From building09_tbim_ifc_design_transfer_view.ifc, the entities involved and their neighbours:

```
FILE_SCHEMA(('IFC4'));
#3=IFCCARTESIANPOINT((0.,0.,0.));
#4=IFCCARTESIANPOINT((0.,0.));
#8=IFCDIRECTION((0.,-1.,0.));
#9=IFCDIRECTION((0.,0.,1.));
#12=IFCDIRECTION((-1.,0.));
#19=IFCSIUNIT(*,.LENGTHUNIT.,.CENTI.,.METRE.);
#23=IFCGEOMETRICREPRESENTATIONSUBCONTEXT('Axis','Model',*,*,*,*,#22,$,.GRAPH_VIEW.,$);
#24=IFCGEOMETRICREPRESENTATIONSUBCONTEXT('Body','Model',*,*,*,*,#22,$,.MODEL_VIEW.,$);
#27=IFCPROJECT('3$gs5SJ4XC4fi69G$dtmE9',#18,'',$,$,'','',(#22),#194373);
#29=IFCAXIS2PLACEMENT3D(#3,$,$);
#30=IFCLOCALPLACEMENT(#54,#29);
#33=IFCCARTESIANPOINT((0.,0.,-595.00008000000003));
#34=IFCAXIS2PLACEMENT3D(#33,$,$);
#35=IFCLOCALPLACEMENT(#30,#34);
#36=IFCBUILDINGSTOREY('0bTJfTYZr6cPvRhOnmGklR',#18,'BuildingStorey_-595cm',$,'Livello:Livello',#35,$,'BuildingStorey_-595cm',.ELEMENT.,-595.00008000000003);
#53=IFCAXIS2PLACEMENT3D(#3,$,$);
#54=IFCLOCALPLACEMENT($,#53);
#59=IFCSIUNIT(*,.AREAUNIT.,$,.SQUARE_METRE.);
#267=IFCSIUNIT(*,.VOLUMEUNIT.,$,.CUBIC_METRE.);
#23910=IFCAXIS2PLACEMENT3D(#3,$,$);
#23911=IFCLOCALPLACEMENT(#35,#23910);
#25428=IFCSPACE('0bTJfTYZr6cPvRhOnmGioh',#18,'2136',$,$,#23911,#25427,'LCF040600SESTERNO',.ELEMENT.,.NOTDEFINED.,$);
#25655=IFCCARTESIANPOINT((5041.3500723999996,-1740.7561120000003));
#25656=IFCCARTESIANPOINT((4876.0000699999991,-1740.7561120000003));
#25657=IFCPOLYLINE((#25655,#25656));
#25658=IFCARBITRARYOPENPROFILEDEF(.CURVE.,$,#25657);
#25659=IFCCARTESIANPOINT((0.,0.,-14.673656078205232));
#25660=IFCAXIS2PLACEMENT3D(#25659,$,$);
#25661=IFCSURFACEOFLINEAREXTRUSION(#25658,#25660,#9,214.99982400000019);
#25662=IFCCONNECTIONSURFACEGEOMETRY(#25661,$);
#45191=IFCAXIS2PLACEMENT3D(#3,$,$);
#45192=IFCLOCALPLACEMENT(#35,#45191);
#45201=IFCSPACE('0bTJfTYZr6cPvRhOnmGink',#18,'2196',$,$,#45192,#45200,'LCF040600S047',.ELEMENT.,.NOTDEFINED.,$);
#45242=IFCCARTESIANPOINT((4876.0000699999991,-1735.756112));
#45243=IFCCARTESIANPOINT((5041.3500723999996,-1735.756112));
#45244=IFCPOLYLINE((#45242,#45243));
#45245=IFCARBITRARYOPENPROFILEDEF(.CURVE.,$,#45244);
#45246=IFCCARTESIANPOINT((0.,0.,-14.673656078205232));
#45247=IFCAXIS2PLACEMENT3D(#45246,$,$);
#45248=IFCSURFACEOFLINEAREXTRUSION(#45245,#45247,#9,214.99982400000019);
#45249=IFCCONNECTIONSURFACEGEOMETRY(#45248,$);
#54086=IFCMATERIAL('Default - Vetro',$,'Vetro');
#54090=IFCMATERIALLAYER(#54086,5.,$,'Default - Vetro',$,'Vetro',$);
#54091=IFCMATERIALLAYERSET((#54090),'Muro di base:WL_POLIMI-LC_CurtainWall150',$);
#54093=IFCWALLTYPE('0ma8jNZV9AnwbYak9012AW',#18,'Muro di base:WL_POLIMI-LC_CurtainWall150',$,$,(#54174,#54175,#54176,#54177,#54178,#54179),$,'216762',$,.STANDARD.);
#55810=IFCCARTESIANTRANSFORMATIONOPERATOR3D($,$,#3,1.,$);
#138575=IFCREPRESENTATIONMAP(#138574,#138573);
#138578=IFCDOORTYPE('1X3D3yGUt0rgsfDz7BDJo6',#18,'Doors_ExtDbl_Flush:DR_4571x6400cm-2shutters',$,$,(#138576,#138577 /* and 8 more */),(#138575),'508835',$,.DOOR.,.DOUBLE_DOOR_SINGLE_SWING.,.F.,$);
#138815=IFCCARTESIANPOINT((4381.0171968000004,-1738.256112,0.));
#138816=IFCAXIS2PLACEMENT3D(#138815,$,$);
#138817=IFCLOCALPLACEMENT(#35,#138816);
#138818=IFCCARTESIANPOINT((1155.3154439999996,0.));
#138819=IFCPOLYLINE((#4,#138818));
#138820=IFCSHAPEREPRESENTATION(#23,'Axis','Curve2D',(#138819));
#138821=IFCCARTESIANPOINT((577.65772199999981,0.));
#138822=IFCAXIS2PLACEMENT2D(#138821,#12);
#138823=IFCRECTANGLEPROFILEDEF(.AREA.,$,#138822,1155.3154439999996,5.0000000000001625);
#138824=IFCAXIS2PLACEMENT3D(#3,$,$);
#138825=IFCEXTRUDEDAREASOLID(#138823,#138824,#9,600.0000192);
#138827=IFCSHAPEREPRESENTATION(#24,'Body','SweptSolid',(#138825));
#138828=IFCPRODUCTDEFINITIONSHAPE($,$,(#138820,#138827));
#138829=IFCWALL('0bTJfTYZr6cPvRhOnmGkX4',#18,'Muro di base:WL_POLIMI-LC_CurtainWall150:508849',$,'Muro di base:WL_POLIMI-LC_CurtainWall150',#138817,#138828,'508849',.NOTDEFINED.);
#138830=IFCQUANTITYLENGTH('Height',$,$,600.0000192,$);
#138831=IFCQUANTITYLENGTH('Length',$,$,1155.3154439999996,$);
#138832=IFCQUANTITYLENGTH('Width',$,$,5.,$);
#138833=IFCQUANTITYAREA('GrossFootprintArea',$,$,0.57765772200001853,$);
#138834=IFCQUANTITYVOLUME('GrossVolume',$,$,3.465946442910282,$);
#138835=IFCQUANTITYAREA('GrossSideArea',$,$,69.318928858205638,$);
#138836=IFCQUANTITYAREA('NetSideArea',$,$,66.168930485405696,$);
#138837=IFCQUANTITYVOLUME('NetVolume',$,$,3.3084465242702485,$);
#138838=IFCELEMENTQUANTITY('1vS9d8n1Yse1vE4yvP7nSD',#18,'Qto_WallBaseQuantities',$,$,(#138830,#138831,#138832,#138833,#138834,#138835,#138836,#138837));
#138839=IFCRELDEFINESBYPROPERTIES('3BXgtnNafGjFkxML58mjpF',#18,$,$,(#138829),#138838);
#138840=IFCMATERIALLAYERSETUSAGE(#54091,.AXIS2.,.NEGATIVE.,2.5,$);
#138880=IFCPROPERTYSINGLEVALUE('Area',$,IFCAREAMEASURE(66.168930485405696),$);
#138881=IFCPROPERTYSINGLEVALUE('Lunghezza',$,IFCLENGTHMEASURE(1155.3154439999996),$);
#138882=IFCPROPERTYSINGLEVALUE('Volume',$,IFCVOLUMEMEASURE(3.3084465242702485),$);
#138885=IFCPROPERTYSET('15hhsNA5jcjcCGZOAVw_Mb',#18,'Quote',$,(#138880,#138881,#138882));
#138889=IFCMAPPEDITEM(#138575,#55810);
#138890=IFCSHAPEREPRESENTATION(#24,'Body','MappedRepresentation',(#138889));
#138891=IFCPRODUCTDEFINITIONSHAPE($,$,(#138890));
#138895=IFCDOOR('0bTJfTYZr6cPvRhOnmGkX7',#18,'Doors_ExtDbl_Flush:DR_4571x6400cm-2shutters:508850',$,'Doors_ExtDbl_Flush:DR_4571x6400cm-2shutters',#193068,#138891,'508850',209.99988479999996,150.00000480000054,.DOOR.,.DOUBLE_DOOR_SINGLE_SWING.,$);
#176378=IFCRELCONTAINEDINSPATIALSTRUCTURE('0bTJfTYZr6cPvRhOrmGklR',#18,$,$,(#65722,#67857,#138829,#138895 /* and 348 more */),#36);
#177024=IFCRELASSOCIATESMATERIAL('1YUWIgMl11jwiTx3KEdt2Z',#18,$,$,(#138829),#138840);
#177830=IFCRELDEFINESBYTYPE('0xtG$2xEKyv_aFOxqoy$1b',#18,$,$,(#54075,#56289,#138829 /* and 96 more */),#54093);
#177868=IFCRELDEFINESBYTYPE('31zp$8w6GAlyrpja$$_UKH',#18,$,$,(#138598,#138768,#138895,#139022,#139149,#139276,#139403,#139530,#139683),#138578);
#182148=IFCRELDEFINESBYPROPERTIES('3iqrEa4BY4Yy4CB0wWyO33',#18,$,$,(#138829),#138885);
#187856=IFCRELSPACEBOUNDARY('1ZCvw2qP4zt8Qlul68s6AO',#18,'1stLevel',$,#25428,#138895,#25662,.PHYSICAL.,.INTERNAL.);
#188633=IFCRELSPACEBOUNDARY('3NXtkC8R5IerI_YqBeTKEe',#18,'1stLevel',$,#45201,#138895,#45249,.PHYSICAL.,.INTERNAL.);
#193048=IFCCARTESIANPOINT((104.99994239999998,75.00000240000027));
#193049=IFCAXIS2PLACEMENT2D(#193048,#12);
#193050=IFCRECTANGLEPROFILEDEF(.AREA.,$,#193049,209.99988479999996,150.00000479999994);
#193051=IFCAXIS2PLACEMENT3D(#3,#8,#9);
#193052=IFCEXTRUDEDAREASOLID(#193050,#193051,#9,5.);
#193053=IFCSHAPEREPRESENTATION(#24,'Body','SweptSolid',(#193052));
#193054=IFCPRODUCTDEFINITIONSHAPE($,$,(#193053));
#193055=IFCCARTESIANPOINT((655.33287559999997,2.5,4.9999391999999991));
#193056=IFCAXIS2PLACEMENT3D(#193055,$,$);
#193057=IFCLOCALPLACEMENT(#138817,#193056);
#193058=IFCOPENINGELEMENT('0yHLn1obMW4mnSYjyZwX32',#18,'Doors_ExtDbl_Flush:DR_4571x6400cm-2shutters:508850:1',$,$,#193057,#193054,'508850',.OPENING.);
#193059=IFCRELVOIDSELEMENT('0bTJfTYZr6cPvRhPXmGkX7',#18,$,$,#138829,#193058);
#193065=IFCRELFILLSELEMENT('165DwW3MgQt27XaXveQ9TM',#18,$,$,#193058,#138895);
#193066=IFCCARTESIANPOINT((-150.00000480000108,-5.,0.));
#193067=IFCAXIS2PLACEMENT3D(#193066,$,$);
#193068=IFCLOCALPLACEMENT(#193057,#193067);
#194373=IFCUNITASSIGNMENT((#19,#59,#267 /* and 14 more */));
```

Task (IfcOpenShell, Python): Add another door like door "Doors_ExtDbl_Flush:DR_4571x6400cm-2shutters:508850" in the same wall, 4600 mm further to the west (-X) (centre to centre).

```python
import numpy as np
import ifcopenshell
import ifcopenshell.api.feature
import ifcopenshell.api.geometry
import ifcopenshell.api.pset
import ifcopenshell.api.root
import ifcopenshell.geom
import ifcopenshell.util.element
import ifcopenshell.util.placement
import ifcopenshell.util.shape
import ifcopenshell.util.unit

model = ifcopenshell.open("building09_tbim_ifc_design_transfer_view.ifc")
unit_scale = ifcopenshell.util.unit.calculate_unit_scale(model)
area_scale = ifcopenshell.util.unit.calculate_unit_scale(model, "AREAUNIT")
volume_scale = ifcopenshell.util.unit.calculate_unit_scale(model, "VOLUMEUNIT")
settings = ifcopenshell.geom.settings()


def volume(element):
    """Net volume in cubic metres, openings subtracted."""
    shape = ifcopenshell.geom.create_shape(settings, element)
    return ifcopenshell.util.shape.get_volume(shape.geometry)


def reuse_history(source, copy):
    """copy_class also copies each property set's owner history, people and application; keep the originals."""
    for rel in copy.IsDefinedBy:
        if rel.is_a("IfcRelDefinesByProperties") and (history := rel.RelatingPropertyDefinition.OwnerHistory):
            rel.RelatingPropertyDefinition.OwnerHistory = source.OwnerHistory
            ifcopenshell.util.element.remove_deep2(model, history)


door = model.by_guid("0bTJfTYZr6cPvRhOnmGkX7")
opening = door.FillsVoids[0].RelatingOpeningElement
wall = opening.VoidsElements[0].RelatingBuildingElement
before = volume(wall)
shift = ifcopenshell.util.placement.get_local_placement(wall.ObjectPlacement)[:3, 0] * -4.6 / unit_scale

# copy_class copies the void relationship, type, container and properties, but no geometry.
new_opening = ifcopenshell.api.root.copy_class(model, product=opening)
new_opening.Representation = ifcopenshell.util.element.copy_deep(
    model, opening.Representation, exclude=["IfcGeometricRepresentationContext", "IfcRepresentationMap"]
)
new_opening.Name = "Doors_ExtDbl_Flush:DR_4571x6400cm-2shutters"
new_opening.Tag = None
reuse_history(opening, new_opening)
new_door = ifcopenshell.api.root.copy_class(model, product=door)
new_door.Representation = ifcopenshell.util.element.copy_deep(
    model, door.Representation, exclude=["IfcGeometricRepresentationContext", "IfcRepresentationMap"]
)
new_door.Name = "Doors_ExtDbl_Flush:DR_4571x6400cm-2shutters"
new_door.Tag = None
reuse_history(door, new_door)
ifcopenshell.api.feature.add_filling(model, opening=new_opening, element=new_door)

for old, new in ((opening, new_opening), (door, new_door)):
    matrix = ifcopenshell.util.placement.get_local_placement(old.ObjectPlacement)
    matrix[:3, 3] += shift
    ifcopenshell.api.geometry.edit_object_placement(model, product=new, matrix=matrix, is_si=False)

# The copied space boundaries still share their surfaces with the original.
for rel in new_door.ProvidesBoundaries:
    if rel.ConnectionGeometry:
        rel.ConnectionGeometry = ifcopenshell.util.element.copy_deep(model, rel.ConnectionGeometry)

# Space boundary surfaces are stored in each space's coordinates; move them too.
for rel in new_door.ProvidesBoundaries:
    if not rel.ConnectionGeometry:
        continue
    surface = rel.ConnectionGeometry.SurfaceOnRelatingElement
    space_matrix = ifcopenshell.util.placement.get_local_placement(rel.RelatingSpace.ObjectPlacement)
    point = np.array(surface.Position.Location.Coordinates) + space_matrix[:3, :3].T @ shift
    surface.Position = model.createIfcAxis2Placement3D(
        model.createIfcCartesianPoint(point.tolist()), surface.Position.Axis, surface.Position.RefDirection
    )

after = volume(wall)
thickness = 0.05  # wall thickness in metres

# Update the wall's stored quantities.
qto = model.by_id(ifcopenshell.util.element.get_pset(wall, "Qto_WallBaseQuantities", should_inherit=False)["id"])
ifcopenshell.api.pset.edit_qto(model, qto=qto, properties={
    "NetSideArea": after / thickness / area_scale,
    "NetVolume": after / volume_scale,
})
pset = model.by_id(ifcopenshell.util.element.get_pset(wall, "Quote", should_inherit=False)["id"])
ifcopenshell.api.pset.edit_pset(model, pset=pset, properties={
    "Area": model.create_entity("IfcAreaMeasure", after / thickness / area_scale),
    "Volume": model.create_entity("IfcVolumeMeasure", after / volume_scale),
})

print(f"wall volume {before:.3f} -> {after:.3f} m3")

model.write("building09_tbim_ifc_design_transfer_view-out.ifc")
```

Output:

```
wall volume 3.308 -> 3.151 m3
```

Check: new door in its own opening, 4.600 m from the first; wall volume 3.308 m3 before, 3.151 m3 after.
